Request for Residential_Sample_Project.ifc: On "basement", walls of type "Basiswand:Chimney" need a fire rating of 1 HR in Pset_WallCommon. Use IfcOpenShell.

First a look at what the model holds.

```python
import ifcopenshell
import ifcopenshell.util.element

model = ifcopenshell.open("Residential_Sample_Project.ifc")
print(model.schema)
storey = next(s for s in model.by_type("IfcBuildingStorey") if s.Name == "basement")
walls = [e for e in ifcopenshell.util.element.get_decomposition(storey) if e.is_a("IfcWall")]
seen = {}
for e in walls:
    element_type = ifcopenshell.util.element.get_type(e)
    key = (element_type.Name if element_type != e and element_type else None, ifcopenshell.util.element.get_pset(e, "Pset_WallCommon", "FireRating"))
    seen[key] = seen.get(key, 0) + 1
for (name, value), count in sorted(seen.items(), key=str):
    print(count, "x", name, "|", value)
```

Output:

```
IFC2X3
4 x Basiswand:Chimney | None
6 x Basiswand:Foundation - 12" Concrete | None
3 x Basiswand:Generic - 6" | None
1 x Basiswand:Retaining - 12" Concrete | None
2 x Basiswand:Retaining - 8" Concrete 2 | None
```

```python
import ifcopenshell
import ifcopenshell.api.pset
import ifcopenshell.util.element

model = ifcopenshell.open("Residential_Sample_Project.ifc")

storey = next(s for s in model.by_type("IfcBuildingStorey") if s.Name == "basement")
walls = [e for e in ifcopenshell.util.element.get_decomposition(storey) if e.is_a("IfcWall")]

count = 0
for e in walls:
    element_type = ifcopenshell.util.element.get_type(e)
    if element_type in (None, e) or element_type.Name != "Basiswand:Chimney":
        continue
    # add_pset returns the element's existing set when there is one.
    pset = ifcopenshell.api.pset.add_pset(model, product=e, name="Pset_WallCommon")
    ifcopenshell.api.pset.edit_pset(model, pset=pset, properties={"FireRating": "1 HR"})
    count += 1

print(count, "walls updated")

model.write("Residential_Sample_Project_rev.ifc")
```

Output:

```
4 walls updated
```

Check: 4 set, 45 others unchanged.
